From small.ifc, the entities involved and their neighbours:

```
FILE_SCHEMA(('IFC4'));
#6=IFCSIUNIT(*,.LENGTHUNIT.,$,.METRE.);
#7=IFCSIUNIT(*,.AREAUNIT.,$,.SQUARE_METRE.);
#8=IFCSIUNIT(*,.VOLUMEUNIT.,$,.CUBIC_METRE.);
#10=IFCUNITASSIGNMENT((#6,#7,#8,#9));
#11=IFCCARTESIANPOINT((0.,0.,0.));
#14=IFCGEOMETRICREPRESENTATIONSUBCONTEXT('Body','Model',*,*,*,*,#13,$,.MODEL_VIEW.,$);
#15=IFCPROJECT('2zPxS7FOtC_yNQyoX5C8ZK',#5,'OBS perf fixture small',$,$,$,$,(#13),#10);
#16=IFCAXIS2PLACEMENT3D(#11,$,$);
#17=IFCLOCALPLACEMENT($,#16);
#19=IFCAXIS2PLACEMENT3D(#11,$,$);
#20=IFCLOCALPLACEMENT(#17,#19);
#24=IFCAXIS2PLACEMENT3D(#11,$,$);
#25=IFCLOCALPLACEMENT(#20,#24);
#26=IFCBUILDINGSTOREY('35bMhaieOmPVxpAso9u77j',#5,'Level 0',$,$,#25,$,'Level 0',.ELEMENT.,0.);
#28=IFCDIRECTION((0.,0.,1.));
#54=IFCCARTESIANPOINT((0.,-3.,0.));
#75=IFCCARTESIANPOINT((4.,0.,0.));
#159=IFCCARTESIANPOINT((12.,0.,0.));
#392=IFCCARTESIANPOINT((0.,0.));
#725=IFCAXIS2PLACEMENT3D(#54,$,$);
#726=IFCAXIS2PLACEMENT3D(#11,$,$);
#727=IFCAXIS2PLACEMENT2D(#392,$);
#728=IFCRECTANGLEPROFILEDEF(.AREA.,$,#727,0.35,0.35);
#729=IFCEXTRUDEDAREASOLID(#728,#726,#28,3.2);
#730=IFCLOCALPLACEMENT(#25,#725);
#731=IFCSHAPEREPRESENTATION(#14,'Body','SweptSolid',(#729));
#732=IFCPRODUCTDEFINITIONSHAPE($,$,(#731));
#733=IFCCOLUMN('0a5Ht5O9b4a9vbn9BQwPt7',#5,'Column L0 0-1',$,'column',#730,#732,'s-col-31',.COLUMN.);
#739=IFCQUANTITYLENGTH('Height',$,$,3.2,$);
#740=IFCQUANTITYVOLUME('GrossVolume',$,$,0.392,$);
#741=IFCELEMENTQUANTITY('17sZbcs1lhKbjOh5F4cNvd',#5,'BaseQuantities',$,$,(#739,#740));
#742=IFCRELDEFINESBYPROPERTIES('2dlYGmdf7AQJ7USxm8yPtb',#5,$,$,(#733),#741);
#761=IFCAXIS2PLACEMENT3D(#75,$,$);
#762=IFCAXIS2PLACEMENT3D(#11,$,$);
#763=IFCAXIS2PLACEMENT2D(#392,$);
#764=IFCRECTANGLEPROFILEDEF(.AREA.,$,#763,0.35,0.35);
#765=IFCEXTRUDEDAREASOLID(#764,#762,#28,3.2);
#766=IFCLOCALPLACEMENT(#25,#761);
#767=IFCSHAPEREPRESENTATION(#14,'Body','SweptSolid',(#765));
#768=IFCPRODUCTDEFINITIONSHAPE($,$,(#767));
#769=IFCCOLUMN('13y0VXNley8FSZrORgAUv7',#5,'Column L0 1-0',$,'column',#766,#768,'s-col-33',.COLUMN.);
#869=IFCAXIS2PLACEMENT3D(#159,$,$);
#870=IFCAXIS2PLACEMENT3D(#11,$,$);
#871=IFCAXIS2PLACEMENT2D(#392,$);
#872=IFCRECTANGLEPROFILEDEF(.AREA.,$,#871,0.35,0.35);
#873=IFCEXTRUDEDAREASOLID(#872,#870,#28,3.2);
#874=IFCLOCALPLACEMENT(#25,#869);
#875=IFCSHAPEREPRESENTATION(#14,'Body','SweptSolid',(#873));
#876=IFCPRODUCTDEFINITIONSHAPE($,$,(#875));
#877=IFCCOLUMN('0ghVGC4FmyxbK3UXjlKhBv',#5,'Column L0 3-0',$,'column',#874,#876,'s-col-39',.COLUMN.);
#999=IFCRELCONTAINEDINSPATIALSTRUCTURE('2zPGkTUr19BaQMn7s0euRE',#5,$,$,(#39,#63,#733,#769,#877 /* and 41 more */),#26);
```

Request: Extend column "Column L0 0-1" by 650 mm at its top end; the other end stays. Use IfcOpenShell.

```python
import ifcopenshell
import ifcopenshell.api.pset
import ifcopenshell.util.element
import ifcopenshell.util.representation
import ifcopenshell.util.unit

model = ifcopenshell.open("small.ifc")
unit_scale = ifcopenshell.util.unit.calculate_unit_scale(model)

member = model.by_id(733)
change = 0.65 / unit_scale

# The extrusion runs towards the end named, so only its depth changes.
body = ifcopenshell.util.representation.get_representation(member, "Model", "Body")
solid = body.Items[0]
old_length = solid.Depth
solid.Depth += change

# Update the stored length and volume.
qto = model.by_id(ifcopenshell.util.element.get_pset(member, "BaseQuantities", should_inherit=False)["id"])
ifcopenshell.api.pset.edit_qto(model, qto=qto, properties={
    "Height": solid.Depth,
    "GrossVolume": ifcopenshell.util.element.get_pset(member, "BaseQuantities", "GrossVolume") * solid.Depth / old_length,
})

print(f"length {old_length:g} -> {solid.Depth:g}")

model.write("small_v2.ifc")
```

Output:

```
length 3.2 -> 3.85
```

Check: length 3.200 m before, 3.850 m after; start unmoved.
